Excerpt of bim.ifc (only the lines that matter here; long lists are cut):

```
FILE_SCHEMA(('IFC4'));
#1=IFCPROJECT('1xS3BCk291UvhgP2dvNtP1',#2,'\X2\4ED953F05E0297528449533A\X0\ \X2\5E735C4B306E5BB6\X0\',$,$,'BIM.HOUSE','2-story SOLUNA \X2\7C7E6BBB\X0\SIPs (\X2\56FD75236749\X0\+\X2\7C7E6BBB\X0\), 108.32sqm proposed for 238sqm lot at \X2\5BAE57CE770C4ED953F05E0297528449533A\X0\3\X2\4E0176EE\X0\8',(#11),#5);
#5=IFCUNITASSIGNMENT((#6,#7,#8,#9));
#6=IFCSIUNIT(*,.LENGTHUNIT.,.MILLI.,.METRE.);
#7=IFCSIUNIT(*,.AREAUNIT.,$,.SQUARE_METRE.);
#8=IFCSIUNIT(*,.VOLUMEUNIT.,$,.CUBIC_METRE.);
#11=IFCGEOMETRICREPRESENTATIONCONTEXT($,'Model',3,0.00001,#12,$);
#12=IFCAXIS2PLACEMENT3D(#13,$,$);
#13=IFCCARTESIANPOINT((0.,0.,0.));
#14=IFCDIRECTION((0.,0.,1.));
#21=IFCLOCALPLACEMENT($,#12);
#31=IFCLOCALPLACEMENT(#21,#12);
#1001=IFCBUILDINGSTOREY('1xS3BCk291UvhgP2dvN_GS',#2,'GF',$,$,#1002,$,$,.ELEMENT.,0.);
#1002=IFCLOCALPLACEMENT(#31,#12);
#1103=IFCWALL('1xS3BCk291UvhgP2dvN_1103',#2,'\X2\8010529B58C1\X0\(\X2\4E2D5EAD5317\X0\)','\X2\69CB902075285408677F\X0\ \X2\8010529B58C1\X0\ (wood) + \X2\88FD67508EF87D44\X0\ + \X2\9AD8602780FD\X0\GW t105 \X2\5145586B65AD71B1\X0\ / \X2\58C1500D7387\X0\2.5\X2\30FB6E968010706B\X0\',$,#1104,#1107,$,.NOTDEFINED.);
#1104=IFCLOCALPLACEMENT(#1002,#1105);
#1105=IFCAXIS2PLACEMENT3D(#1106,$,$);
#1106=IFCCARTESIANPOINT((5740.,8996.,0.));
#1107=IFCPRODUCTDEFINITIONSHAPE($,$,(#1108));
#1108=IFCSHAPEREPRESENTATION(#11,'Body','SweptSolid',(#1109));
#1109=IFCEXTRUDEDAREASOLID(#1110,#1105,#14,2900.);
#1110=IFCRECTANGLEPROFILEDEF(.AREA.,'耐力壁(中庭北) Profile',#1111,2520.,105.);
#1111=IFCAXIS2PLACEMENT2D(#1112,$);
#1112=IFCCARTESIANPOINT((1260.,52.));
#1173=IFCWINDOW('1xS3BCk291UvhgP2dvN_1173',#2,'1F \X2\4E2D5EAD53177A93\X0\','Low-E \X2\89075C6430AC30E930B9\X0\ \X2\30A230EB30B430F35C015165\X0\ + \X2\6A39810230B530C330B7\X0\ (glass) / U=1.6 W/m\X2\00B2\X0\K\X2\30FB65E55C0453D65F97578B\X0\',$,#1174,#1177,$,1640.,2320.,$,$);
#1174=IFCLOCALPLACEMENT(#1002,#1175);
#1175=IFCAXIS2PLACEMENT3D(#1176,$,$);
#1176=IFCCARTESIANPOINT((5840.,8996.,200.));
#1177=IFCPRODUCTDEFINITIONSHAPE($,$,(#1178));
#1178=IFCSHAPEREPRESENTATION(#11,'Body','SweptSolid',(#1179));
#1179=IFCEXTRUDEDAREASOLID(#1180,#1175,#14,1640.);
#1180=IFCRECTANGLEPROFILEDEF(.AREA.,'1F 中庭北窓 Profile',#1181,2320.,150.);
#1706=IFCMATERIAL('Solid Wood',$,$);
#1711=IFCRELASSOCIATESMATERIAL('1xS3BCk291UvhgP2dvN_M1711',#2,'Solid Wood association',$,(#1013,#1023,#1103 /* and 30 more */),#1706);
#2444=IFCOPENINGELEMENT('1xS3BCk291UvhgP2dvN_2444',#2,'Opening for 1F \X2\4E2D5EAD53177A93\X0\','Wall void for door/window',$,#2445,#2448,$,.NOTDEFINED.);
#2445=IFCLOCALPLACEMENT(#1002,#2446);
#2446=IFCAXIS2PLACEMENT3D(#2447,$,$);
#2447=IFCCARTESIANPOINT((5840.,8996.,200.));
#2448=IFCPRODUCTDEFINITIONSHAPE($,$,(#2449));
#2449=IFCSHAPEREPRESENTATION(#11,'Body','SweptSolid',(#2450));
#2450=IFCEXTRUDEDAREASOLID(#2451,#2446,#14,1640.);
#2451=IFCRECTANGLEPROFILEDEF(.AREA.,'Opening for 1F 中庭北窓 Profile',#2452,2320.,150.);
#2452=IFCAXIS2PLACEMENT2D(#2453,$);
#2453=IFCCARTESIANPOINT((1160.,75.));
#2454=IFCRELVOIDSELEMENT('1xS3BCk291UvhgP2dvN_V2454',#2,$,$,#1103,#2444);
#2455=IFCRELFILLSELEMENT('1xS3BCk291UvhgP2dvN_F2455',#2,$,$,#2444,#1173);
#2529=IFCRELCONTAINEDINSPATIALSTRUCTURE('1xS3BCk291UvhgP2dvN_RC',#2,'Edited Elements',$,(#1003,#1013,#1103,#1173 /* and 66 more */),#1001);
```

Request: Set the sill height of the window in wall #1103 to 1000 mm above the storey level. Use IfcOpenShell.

```python
import numpy as np
import ifcopenshell
import ifcopenshell.api.geometry
import ifcopenshell.geom
import ifcopenshell.util.element
import ifcopenshell.util.placement
import ifcopenshell.util.shape
import ifcopenshell.util.unit

model = ifcopenshell.open("bim.ifc")
unit_scale = ifcopenshell.util.unit.calculate_unit_scale(model)

window = model.by_id(1173)
opening = window.FillsVoids[0].RelatingOpeningElement
storey = ifcopenshell.util.element.get_container(window, ifc_class="IfcBuildingStorey")
level = ifcopenshell.util.placement.get_local_placement(storey.ObjectPlacement)[2, 3]

# The opening's origin need not be at the sill, so measure its lowest point.
shape = ifcopenshell.geom.create_shape(ifcopenshell.geom.settings(), opening)
bottom = ifcopenshell.util.shape.get_shape_bottom_elevation(shape, shape.geometry) / unit_scale
dz = level + 1 / unit_scale - bottom

shift = np.array([0.0, 0.0, dz])
# The window is not placed relative to its opening, so move both.
for product in (opening, window):
    matrix = ifcopenshell.util.placement.get_local_placement(product.ObjectPlacement)
    matrix[:3, 3] += shift
    ifcopenshell.api.geometry.edit_object_placement(model, product=product, matrix=matrix, is_si=False)

print(f"moved by {dz * unit_scale:+.3f} m")

model.write("bim_rev.ifc")
```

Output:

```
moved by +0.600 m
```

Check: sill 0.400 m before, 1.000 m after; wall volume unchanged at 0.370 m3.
